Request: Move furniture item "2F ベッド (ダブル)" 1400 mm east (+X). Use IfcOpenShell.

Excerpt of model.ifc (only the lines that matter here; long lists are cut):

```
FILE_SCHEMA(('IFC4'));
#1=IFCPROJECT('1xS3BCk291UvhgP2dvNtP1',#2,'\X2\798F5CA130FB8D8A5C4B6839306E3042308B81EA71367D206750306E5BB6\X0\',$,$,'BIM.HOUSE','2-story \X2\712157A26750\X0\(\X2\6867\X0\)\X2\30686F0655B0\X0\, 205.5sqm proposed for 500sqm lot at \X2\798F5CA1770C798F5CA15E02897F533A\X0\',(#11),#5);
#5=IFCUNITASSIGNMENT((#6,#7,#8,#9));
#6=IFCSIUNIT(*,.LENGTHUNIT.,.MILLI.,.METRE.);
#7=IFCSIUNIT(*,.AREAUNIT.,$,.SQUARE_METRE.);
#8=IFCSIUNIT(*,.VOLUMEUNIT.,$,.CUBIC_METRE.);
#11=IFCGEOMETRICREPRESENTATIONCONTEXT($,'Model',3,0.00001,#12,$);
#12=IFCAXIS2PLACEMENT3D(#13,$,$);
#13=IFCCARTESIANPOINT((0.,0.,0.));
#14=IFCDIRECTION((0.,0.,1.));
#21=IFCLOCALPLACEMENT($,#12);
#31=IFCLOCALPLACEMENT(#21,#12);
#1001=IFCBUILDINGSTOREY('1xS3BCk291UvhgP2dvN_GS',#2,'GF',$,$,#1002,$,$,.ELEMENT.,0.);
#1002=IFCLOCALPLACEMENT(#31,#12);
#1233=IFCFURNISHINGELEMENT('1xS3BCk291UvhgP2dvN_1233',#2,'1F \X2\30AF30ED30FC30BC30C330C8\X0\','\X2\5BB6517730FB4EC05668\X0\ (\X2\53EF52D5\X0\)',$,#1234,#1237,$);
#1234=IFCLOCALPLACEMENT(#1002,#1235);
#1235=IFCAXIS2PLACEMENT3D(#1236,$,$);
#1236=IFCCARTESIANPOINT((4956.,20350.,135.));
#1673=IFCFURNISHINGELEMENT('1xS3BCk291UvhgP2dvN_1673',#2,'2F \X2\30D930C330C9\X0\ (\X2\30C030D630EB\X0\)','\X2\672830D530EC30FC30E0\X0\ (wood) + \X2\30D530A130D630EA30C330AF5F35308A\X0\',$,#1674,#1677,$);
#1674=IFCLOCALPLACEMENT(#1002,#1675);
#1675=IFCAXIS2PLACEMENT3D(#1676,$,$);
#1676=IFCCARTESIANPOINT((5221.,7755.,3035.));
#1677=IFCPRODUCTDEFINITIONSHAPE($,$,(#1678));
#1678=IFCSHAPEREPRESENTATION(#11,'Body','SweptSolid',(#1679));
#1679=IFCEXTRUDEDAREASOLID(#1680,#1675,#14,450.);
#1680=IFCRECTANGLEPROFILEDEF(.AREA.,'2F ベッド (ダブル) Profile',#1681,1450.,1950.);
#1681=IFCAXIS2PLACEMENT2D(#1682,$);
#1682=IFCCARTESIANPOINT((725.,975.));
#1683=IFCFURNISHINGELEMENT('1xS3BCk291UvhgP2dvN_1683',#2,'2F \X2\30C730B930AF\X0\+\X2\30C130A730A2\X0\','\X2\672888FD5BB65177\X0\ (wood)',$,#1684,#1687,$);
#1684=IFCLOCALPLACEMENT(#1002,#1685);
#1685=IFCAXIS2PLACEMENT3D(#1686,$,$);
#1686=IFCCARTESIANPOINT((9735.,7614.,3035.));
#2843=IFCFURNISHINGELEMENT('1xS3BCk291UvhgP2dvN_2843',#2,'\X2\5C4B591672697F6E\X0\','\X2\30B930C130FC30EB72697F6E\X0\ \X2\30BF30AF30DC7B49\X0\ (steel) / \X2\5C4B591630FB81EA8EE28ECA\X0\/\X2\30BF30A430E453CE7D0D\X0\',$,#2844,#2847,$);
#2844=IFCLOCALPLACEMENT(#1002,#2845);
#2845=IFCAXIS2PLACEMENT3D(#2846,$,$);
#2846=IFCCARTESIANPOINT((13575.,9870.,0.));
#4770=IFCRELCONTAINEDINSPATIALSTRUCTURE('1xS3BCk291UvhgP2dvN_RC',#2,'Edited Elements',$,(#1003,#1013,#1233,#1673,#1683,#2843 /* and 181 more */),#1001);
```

```python
import ifcopenshell
import ifcopenshell.api.geometry
import ifcopenshell.util.placement

model = ifcopenshell.open("model.ifc")

item = model.by_id(1673)
matrix = ifcopenshell.util.placement.get_local_placement(item.ObjectPlacement)
matrix[0, 3] += 1400.0
ifcopenshell.api.geometry.edit_object_placement(model, product=item, matrix=matrix, is_si=False)

print(ifcopenshell.util.placement.get_local_placement(item.ObjectPlacement).round(3) + 0.0)

model.write("model-out.ifc")
```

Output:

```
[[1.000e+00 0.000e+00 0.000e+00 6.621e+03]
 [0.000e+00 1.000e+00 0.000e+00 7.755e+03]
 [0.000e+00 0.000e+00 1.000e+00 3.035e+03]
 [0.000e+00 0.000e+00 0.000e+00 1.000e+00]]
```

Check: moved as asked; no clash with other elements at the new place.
